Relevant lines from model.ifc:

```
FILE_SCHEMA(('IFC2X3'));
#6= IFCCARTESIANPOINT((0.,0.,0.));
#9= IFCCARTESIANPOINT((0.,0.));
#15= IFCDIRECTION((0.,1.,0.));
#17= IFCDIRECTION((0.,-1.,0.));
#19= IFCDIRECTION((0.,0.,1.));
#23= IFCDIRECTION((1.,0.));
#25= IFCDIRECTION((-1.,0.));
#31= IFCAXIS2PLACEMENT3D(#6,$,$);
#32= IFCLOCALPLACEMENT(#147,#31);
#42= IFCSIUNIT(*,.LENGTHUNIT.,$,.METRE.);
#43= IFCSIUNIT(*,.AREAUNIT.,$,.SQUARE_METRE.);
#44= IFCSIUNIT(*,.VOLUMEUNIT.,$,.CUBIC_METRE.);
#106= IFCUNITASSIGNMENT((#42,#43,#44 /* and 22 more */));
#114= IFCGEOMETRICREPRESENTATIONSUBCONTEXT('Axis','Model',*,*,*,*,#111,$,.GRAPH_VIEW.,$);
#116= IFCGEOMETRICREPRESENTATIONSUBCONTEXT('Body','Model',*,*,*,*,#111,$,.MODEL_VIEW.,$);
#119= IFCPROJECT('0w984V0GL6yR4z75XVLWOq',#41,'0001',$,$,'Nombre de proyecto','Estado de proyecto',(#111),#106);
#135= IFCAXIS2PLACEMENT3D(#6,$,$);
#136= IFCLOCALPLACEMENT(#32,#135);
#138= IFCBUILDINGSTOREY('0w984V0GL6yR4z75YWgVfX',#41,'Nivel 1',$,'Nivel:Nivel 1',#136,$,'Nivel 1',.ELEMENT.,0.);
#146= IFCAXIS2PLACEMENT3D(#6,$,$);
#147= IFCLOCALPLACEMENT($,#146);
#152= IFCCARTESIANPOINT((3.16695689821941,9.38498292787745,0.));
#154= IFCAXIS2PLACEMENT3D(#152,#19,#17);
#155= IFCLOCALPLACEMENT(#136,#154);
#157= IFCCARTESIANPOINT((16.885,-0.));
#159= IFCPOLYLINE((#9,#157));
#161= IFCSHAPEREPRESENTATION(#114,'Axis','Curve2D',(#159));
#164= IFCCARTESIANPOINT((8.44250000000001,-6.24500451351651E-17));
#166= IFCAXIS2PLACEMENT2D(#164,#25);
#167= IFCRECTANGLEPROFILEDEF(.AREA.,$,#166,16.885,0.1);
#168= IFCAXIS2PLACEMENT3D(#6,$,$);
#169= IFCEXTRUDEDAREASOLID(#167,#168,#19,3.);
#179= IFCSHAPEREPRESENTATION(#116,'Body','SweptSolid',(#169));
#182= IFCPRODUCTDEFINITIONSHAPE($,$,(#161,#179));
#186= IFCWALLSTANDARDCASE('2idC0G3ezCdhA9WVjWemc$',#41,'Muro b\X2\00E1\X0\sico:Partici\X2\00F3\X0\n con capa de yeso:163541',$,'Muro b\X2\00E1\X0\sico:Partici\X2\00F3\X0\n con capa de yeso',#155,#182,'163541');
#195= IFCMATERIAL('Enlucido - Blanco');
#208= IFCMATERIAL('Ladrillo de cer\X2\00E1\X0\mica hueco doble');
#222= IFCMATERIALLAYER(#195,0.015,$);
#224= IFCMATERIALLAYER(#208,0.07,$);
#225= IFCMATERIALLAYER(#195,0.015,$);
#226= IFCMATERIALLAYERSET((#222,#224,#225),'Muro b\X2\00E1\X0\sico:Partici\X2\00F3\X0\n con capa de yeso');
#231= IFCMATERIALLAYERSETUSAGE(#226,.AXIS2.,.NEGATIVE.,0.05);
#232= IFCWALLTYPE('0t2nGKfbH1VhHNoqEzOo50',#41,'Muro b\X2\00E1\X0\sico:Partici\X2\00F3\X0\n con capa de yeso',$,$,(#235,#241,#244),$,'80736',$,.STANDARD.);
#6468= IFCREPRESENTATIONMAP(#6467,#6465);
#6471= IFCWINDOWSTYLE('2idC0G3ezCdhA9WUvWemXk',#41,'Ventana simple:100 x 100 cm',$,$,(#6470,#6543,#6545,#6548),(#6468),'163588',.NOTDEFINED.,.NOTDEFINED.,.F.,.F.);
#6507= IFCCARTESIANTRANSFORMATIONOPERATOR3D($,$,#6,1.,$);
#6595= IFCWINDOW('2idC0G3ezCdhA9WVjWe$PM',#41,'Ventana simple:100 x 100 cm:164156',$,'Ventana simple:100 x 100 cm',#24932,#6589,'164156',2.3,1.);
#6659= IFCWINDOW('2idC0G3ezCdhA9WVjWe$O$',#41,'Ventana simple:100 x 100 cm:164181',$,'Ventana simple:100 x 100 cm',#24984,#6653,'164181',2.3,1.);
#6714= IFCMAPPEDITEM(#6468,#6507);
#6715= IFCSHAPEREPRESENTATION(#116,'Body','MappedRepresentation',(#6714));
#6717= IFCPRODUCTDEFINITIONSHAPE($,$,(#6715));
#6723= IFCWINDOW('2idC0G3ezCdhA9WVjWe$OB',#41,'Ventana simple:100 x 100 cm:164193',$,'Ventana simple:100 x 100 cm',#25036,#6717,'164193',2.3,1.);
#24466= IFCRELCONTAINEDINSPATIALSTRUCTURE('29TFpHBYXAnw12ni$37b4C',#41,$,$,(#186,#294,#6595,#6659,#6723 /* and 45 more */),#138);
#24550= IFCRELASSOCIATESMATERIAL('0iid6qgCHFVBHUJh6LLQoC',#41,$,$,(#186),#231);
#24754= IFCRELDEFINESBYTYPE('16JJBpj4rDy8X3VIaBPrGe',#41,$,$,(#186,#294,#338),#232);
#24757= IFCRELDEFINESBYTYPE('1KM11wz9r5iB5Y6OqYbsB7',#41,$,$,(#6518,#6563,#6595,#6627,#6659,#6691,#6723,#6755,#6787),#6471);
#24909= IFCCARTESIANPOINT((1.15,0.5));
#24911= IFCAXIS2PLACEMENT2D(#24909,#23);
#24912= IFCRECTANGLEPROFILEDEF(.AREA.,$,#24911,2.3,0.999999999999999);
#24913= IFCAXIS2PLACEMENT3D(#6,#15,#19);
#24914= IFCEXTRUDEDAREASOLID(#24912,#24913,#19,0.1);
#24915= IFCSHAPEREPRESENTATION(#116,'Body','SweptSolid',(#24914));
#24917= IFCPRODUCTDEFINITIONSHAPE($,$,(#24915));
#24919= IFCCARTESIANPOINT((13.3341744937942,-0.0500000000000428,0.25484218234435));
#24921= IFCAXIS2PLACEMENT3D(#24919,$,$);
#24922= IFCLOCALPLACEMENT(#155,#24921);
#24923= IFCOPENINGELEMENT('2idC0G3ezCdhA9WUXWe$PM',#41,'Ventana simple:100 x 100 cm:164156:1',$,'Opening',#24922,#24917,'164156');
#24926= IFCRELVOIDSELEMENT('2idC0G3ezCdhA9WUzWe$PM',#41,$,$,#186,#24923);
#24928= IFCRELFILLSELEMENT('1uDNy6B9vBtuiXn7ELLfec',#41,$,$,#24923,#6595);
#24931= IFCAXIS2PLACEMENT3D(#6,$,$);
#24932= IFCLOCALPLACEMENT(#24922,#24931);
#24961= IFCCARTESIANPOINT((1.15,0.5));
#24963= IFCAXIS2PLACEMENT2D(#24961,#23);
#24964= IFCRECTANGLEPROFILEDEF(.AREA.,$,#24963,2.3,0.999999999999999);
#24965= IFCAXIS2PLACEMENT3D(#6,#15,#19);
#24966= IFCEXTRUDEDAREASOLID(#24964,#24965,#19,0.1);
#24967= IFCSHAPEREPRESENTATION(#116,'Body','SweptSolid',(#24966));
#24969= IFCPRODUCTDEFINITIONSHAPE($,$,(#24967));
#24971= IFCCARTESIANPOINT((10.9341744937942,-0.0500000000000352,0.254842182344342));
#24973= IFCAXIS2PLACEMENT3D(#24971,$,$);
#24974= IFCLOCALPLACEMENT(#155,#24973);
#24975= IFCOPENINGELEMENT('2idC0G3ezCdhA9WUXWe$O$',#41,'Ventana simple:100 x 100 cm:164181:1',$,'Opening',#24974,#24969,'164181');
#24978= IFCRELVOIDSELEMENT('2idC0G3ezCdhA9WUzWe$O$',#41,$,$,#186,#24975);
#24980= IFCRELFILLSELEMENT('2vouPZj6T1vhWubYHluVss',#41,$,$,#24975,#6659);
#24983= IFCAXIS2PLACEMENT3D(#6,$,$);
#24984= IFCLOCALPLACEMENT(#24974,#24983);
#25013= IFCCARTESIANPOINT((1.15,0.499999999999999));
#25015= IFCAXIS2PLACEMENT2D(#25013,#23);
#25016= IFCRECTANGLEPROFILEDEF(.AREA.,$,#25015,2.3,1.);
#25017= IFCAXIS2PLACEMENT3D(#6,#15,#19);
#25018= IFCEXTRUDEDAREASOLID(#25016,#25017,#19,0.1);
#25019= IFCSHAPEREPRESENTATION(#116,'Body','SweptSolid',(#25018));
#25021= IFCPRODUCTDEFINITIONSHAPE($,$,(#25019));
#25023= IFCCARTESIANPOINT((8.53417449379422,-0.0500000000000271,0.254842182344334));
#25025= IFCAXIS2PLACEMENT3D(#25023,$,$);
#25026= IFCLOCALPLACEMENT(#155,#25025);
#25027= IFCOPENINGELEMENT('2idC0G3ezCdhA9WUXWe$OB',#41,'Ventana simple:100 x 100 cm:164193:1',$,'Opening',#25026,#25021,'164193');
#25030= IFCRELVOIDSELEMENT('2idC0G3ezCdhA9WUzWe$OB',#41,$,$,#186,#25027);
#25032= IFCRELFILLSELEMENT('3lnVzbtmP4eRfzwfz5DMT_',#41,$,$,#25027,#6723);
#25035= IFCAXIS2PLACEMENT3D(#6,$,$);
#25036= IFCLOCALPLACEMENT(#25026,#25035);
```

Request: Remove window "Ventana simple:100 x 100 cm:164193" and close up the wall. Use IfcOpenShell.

```python
import ifcopenshell
import ifcopenshell.api.feature
import ifcopenshell.api.root
import ifcopenshell.geom
import ifcopenshell.util.shape

model = ifcopenshell.open("model.ifc")
settings = ifcopenshell.geom.settings()


def volume(element):
    """Net volume in cubic metres, openings subtracted."""
    shape = ifcopenshell.geom.create_shape(settings, element)
    return ifcopenshell.util.shape.get_volume(shape.geometry)


window = model.by_guid("2idC0G3ezCdhA9WVjWe$OB")
opening = window.FillsVoids[0].RelatingOpeningElement
wall = opening.VoidsElements[0].RelatingBuildingElement
before = volume(wall)

ifcopenshell.api.root.remove_product(model, product=window)
ifcopenshell.api.feature.remove_feature(model, feature=opening)

after = volume(wall)

print(f"wall volume {before:.3f} -> {after:.3f} m3")

model.write("model_v2.ifc")
```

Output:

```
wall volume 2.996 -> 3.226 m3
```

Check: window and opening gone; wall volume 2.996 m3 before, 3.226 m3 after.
